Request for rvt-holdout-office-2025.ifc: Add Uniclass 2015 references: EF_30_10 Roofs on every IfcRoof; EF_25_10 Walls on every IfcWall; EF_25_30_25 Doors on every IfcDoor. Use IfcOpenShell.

First a look at what the model holds.

```python
import ifcopenshell

model = ifcopenshell.open("rvt-holdout-office-2025.ifc")
print(model.schema)
print("classifications:", [c.Name for c in model.by_type("IfcClassification")])
for ifc_class in ("IfcDoor", "IfcRoof", "IfcStair", "IfcWall", "IfcWindow"):
    print(ifc_class, len(model.by_type(ifc_class)))
```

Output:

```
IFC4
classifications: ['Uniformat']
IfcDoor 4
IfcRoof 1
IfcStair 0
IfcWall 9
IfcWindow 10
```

```python
import ifcopenshell
import ifcopenshell.api.classification

model = ifcopenshell.open("rvt-holdout-office-2025.ifc")

system = ifcopenshell.api.classification.add_classification(model, classification="Uniclass 2015")

codes = {
    "IfcRoof": ("EF_30_10", "Roofs"),
    "IfcWall": ("EF_25_10", "Walls"),
    "IfcDoor": ("EF_25_30_25", "Doors"),
}
for ifc_class, (code, name) in codes.items():
    products = model.by_type(ifc_class)
    ifcopenshell.api.classification.add_reference(
        model, products=products, classification=system, identification=code, name=name
    )
    print(code, len(products))

model.write("rvt-holdout-office-2025_rev.ifc")
```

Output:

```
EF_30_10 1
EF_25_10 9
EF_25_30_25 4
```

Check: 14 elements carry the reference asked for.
